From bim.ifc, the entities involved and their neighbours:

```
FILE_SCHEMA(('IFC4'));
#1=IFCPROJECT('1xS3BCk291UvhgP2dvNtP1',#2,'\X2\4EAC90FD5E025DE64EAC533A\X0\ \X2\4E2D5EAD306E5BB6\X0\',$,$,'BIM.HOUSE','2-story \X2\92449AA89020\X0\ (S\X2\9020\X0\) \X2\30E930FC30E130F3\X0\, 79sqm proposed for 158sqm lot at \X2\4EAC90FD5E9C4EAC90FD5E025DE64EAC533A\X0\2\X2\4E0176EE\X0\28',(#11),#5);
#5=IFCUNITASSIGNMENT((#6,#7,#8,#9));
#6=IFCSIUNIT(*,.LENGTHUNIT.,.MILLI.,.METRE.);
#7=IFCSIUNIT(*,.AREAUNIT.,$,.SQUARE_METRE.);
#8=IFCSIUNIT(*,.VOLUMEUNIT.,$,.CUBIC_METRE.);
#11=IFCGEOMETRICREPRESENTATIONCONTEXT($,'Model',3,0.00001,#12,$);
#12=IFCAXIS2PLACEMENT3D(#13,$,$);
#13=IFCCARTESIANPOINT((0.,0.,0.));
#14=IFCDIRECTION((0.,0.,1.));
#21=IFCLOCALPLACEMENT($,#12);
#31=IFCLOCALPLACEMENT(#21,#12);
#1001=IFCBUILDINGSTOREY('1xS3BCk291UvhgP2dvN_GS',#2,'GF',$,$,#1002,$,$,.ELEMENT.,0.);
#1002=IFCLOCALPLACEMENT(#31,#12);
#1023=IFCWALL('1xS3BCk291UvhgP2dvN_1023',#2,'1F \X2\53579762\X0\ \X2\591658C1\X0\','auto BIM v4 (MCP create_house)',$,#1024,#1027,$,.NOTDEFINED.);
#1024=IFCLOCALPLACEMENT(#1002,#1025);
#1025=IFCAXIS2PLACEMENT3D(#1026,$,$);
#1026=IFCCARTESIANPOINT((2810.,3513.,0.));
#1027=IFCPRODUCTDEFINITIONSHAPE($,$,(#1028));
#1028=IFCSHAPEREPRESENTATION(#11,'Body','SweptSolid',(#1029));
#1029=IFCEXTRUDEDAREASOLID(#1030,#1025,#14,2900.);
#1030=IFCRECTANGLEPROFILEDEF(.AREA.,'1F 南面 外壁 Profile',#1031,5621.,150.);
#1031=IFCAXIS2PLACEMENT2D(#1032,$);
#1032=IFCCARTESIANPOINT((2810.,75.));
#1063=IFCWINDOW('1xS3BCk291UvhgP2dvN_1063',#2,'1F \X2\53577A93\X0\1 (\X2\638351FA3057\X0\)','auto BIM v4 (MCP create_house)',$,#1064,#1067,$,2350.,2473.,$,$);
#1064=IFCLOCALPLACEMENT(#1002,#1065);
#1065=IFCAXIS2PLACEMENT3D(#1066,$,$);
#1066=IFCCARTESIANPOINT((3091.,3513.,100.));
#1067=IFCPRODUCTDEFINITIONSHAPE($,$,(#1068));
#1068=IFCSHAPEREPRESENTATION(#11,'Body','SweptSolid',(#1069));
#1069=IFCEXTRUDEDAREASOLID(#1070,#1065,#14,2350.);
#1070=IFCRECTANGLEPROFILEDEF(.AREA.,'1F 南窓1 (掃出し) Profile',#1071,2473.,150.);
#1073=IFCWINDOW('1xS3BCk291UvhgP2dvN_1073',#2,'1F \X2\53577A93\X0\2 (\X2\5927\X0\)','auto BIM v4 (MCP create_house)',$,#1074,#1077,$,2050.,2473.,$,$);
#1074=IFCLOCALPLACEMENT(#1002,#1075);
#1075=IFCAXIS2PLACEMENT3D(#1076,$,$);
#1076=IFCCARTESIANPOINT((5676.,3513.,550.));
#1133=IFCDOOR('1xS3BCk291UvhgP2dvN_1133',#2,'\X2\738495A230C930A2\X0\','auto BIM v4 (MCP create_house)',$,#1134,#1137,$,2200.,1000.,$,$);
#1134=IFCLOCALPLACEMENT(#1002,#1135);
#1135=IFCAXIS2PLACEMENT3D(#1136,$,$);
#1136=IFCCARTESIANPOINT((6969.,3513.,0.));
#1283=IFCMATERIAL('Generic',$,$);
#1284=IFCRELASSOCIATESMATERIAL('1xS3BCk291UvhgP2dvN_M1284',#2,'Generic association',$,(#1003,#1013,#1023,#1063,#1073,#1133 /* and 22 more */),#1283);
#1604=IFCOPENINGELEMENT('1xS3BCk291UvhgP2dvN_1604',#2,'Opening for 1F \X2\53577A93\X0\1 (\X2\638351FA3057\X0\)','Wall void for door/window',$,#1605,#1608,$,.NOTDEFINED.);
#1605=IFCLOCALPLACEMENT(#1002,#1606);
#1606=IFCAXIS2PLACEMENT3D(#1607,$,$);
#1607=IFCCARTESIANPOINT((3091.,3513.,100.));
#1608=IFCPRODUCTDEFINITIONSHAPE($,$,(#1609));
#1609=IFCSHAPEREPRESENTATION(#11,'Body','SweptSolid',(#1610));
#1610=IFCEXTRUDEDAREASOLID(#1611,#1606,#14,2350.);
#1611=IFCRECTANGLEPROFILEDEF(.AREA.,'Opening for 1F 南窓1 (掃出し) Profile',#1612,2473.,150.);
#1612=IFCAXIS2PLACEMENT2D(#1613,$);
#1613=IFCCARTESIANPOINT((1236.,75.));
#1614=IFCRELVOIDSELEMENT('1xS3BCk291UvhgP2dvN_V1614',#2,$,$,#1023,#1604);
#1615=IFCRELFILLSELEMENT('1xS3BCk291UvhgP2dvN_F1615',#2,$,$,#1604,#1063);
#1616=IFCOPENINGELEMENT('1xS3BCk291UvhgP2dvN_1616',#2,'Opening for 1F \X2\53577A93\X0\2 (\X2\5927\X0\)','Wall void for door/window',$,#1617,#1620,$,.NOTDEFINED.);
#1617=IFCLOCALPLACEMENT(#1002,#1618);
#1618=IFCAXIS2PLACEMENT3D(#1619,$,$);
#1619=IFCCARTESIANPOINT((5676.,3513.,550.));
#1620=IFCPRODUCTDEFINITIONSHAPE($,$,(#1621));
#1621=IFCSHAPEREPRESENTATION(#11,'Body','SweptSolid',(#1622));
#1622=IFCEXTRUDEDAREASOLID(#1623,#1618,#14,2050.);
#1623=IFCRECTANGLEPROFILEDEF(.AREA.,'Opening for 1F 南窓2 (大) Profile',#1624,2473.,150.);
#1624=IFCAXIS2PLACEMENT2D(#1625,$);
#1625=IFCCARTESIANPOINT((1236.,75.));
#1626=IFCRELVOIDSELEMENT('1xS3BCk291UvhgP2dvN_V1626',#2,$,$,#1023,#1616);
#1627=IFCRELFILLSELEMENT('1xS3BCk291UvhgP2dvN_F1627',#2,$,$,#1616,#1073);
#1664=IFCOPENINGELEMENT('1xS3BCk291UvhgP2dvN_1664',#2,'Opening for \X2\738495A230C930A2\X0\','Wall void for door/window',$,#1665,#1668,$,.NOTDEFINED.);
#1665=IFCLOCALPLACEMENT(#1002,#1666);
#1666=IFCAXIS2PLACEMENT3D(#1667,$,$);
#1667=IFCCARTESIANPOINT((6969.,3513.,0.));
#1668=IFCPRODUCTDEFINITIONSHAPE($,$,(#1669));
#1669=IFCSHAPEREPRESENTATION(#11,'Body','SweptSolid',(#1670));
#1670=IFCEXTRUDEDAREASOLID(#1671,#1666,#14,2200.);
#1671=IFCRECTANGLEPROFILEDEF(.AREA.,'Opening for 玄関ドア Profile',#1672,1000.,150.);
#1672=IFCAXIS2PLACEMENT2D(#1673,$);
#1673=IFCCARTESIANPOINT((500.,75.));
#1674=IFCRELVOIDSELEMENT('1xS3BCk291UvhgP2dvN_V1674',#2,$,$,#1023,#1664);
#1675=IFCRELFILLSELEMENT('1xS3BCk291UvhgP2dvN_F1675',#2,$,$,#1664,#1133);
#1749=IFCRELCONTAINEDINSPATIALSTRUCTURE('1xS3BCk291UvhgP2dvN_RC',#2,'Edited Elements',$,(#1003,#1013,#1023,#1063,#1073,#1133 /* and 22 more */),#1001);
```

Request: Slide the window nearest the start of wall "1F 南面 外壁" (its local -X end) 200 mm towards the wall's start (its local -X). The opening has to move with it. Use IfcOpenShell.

```python
import ifcopenshell
import ifcopenshell.api.geometry
import ifcopenshell.util.placement
import ifcopenshell.util.unit

model = ifcopenshell.open("bim.ifc")
unit_scale = ifcopenshell.util.unit.calculate_unit_scale(model)

window = model.by_id(1063)
opening = window.FillsVoids[0].RelatingOpeningElement
wall = opening.VoidsElements[0].RelatingBuildingElement

wall_matrix = ifcopenshell.util.placement.get_local_placement(wall.ObjectPlacement)
shift = wall_matrix[:3, 0] * -0.2 / unit_scale
before = ifcopenshell.util.placement.get_local_placement(window.ObjectPlacement)[:3, 3].copy()

# The window is not placed relative to its opening, so move both.
for product in (opening, window):
    matrix = ifcopenshell.util.placement.get_local_placement(product.ObjectPlacement)
    matrix[:3, 3] += shift
    ifcopenshell.api.geometry.edit_object_placement(model, product=product, matrix=matrix, is_si=False)

after = ifcopenshell.util.placement.get_local_placement(window.ObjectPlacement)[:3, 3]
print("window moved by", (after - before).round(3) + 0.0)

model.write("bim_v2.ifc")
```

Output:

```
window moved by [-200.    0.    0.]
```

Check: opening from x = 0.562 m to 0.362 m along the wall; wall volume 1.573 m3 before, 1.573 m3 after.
